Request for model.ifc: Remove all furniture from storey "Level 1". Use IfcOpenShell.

First a look at what the model holds.

```python
import ifcopenshell
import ifcopenshell.util.element

model = ifcopenshell.open("model.ifc")
print(model.schema)
storey = next(s for s in model.by_type("IfcBuildingStorey") if s.Name == "Level 1")
furniture = [e for e in ifcopenshell.util.element.get_decomposition(storey) if e.is_a("IfcFurnishingElement")]
seen = {}
for e in furniture:
    element_type = ifcopenshell.util.element.get_type(e)
    name = element_type.Name if element_type not in (None, e) else None
    seen[name] = seen.get(name, 0) + 1
for name, count in sorted(seen.items(), key=str):
    print(count, "x", name)
```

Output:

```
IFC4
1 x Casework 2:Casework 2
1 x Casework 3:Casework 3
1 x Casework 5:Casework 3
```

```python
import ifcopenshell
import ifcopenshell.api.root
import ifcopenshell.util.element

model = ifcopenshell.open("model.ifc")

storey = next(s for s in model.by_type("IfcBuildingStorey") if s.Name == "Level 1")
furniture = [e for e in ifcopenshell.util.element.get_decomposition(storey) if e.is_a("IfcFurnishingElement")]

for e in furniture:
    ifcopenshell.api.root.remove_product(model, product=e)
print(len(furniture), "removed")

model.write("model-out.ifc")
```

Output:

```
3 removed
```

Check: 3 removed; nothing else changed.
